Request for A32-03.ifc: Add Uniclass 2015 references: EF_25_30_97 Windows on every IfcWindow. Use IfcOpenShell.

First a look at what the model holds.

```python
import ifcopenshell

model = ifcopenshell.open("A32-03.ifc")
print(model.schema)
print("classifications:", [c.Name for c in model.by_type("IfcClassification")])
for ifc_class in ("IfcDoor", "IfcRoof", "IfcStair", "IfcWall", "IfcWindow"):
    print(ifc_class, len(model.by_type(ifc_class)))
```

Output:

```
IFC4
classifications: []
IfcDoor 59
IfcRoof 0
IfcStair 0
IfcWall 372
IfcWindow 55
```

```python
import ifcopenshell
import ifcopenshell.api.classification

model = ifcopenshell.open("A32-03.ifc")

system = ifcopenshell.api.classification.add_classification(model, classification="Uniclass 2015")

codes = {
    "IfcWindow": ("EF_25_30_97", "Windows"),
}
for ifc_class, (code, name) in codes.items():
    products = model.by_type(ifc_class)
    ifcopenshell.api.classification.add_reference(
        model, products=products, classification=system, identification=code, name=name
    )
    print(code, len(products))

model.write("A32-03-out.ifc")
```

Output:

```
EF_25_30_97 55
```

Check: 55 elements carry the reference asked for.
